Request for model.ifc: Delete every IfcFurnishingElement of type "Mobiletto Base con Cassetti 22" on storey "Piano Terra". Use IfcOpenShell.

First a look at what the model holds.

```python
import ifcopenshell
import ifcopenshell.util.element

model = ifcopenshell.open("model.ifc")
print(model.schema)
storey = next(s for s in model.by_type("IfcBuildingStorey") if s.Name == "Piano Terra")
furniture = [e for e in ifcopenshell.util.element.get_decomposition(storey) if e.is_a("IfcFurnishingElement")]
seen = {}
for e in furniture:
    element_type = ifcopenshell.util.element.get_type(e)
    name = element_type.Name if element_type not in (None, e) else None
    seen[name] = seen.get(name, 0) + 1
for name, count in sorted(seen.items(), key=str):
    print(count, "x", name)
```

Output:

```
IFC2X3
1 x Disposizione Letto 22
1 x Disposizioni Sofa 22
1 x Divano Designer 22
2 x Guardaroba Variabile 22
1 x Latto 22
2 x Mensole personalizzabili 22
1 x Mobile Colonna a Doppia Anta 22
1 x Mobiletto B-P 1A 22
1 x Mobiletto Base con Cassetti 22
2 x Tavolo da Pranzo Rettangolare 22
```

```python
import ifcopenshell
import ifcopenshell.api.root
import ifcopenshell.util.element

model = ifcopenshell.open("model.ifc")

storey = next(s for s in model.by_type("IfcBuildingStorey") if s.Name == "Piano Terra")
furniture = [e for e in ifcopenshell.util.element.get_decomposition(storey) if e.is_a("IfcFurnishingElement")]
targets = [e for e in furniture if (t := ifcopenshell.util.element.get_type(e)) not in (None, e) and t.Name == "Mobiletto Base con Cassetti 22"]

for e in targets:
    ifcopenshell.api.root.remove_product(model, product=e)
print(len(targets), "removed")

model.write("model_updated.ifc")
```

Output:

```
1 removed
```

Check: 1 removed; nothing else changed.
